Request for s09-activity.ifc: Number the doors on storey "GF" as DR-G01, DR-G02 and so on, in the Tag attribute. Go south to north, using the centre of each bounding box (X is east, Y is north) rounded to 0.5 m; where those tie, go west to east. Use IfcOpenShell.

First a look at what the model holds.

```python
import ifcopenshell
import ifcopenshell.util.element
import ifcopenshell.util.placement

model = ifcopenshell.open("s09-activity.ifc")
print(model.schema)
storey = next(s for s in model.by_type("IfcBuildingStorey") if s.Name == "GF")
doors = [e for e in ifcopenshell.util.element.get_decomposition(storey) if e.is_a("IfcDoor")]
for e in sorted(doors, key=lambda e: e.id()):
    origin = ifcopenshell.util.placement.get_local_placement(e.ObjectPlacement)[:3, 3]
    print(e.id(), e.Tag, e.Name, origin.round(2) + 0.0, sep=" | ")
```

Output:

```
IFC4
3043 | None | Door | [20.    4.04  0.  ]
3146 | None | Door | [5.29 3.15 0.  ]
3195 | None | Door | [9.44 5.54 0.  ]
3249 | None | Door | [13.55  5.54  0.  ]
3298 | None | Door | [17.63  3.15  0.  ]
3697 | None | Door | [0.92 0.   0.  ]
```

```python
import ifcopenshell
import ifcopenshell.geom
import ifcopenshell.util.element
import ifcopenshell.util.shape

model = ifcopenshell.open("s09-activity.ifc")
settings = ifcopenshell.geom.settings()
settings.set("use-world-coords", True)


def centre(element):
    shape = ifcopenshell.geom.create_shape(settings, element)
    return ifcopenshell.util.shape.get_bbox_centroid(shape.geometry)


storey = next(s for s in model.by_type("IfcBuildingStorey") if s.Name == "GF")
doors = [e for e in ifcopenshell.util.element.get_decomposition(storey) if e.is_a("IfcDoor")]

# Insertion points can sit at a corner or the storey origin, so sort by the geometry (in metres).
centres = {e: centre(e) for e in doors}
doors.sort(key=lambda e: (round(centres[e][1] / 0.5), centres[e][0]))

for i, e in enumerate(doors, start=1):
    number = f"DR-G{i:02d}"
    e.Tag = number
    print(e.id(), number)

model.write("s09-activity_rev.ifc")
```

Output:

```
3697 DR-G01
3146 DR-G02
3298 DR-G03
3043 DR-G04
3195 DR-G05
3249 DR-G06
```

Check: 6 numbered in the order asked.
